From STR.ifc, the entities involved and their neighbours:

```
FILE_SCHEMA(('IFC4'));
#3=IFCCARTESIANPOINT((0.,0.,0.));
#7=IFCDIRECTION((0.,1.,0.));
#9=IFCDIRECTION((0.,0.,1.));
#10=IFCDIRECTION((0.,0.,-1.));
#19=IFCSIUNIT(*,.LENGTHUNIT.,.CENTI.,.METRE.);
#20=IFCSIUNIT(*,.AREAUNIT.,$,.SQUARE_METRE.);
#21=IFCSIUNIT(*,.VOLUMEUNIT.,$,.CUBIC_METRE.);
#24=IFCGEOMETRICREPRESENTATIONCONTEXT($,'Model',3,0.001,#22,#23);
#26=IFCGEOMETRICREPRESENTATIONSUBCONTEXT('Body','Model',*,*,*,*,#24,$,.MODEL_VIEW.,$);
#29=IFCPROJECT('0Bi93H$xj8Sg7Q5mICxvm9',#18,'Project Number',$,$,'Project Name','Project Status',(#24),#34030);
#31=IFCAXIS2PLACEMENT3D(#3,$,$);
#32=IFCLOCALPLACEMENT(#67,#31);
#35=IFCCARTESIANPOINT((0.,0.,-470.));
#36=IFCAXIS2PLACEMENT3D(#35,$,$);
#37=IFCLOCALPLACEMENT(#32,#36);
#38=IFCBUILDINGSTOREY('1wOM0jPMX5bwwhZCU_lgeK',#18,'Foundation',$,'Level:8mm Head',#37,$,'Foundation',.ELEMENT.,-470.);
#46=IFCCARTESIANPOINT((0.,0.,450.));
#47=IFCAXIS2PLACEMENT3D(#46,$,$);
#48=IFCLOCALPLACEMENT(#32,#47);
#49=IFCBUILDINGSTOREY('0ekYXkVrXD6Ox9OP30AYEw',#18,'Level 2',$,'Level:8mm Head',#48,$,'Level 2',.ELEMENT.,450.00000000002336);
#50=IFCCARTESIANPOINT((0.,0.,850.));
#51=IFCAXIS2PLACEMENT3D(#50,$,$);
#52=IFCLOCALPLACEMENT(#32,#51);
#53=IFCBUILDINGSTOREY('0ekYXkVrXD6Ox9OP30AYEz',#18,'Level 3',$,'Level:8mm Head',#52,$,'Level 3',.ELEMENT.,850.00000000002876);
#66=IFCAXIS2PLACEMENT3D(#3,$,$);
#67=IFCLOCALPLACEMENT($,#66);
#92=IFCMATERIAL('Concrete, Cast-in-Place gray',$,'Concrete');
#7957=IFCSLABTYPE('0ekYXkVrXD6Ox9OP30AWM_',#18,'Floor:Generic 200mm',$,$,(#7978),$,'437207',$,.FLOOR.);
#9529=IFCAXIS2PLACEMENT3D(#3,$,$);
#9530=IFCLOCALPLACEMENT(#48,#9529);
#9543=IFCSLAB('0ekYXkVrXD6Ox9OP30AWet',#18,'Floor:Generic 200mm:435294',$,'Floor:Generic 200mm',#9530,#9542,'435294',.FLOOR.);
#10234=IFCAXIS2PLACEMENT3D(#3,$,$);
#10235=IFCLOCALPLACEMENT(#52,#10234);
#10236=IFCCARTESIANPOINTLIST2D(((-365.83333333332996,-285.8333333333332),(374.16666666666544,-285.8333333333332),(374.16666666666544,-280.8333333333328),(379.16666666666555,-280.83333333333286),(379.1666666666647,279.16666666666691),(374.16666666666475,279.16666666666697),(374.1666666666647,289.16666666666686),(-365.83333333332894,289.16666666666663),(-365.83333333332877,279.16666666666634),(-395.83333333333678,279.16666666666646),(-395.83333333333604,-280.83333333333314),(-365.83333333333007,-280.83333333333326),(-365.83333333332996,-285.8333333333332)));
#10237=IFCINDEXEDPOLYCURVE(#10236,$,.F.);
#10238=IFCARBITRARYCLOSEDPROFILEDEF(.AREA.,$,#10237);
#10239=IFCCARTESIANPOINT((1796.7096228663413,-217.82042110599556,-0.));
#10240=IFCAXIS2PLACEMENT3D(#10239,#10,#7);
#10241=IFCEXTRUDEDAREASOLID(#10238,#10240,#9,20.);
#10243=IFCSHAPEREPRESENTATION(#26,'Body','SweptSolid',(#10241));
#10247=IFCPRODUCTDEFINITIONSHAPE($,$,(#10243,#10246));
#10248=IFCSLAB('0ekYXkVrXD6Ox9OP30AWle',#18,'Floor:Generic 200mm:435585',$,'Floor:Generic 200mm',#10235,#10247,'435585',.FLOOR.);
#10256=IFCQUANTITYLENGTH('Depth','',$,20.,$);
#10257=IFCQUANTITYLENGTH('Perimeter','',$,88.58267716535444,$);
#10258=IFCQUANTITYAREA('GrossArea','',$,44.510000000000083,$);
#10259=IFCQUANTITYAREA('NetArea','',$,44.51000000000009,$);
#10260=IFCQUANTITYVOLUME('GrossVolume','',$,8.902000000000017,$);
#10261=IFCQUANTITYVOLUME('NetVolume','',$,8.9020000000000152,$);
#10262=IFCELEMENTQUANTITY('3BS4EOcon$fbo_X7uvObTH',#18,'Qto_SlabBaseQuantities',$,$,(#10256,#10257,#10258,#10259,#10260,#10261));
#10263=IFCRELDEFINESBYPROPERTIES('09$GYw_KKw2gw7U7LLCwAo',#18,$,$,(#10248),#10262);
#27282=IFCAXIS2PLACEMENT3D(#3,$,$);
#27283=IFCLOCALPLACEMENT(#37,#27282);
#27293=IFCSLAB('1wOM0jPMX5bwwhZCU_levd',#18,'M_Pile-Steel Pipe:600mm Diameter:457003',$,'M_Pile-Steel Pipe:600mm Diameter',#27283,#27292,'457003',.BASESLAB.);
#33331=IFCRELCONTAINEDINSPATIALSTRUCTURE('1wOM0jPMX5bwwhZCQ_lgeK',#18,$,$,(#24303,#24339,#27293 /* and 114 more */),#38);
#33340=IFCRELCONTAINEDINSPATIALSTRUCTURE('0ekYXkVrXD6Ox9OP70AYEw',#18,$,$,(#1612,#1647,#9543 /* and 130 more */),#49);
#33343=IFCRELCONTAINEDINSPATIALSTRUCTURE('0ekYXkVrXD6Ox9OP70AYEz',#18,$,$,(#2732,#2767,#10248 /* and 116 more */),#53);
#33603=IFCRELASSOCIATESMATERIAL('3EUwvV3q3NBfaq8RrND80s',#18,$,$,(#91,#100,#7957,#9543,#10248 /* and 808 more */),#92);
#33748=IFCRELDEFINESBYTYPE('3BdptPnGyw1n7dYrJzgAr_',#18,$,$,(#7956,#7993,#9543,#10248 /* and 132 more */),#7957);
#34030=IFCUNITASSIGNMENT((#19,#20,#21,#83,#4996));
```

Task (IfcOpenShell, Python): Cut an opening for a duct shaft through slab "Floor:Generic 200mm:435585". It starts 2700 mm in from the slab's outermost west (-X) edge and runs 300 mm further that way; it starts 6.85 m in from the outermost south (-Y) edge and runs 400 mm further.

```python
import numpy as np
import ifcopenshell
import ifcopenshell.api.feature
import ifcopenshell.api.geometry
import ifcopenshell.api.pset
import ifcopenshell.api.root
import ifcopenshell.geom
import ifcopenshell.util.element
import ifcopenshell.util.placement
import ifcopenshell.util.representation
import ifcopenshell.util.shape
import ifcopenshell.util.unit

model = ifcopenshell.open("STR.ifc")
unit_scale = ifcopenshell.util.unit.calculate_unit_scale(model)
area_scale = ifcopenshell.util.unit.calculate_unit_scale(model, "AREAUNIT")
volume_scale = ifcopenshell.util.unit.calculate_unit_scale(model, "VOLUMEUNIT")
settings = ifcopenshell.geom.settings()


def volume(element):
    """Net volume in cubic metres, openings subtracted."""
    shape = ifcopenshell.geom.create_shape(settings, element)
    return ifcopenshell.util.shape.get_volume(shape.geometry)


slab = model.by_guid("0ekYXkVrXD6Ox9OP30AWle")
before = volume(slab)

# Extent in the slab's own axes, in metres. The edges named are its -X and -Y sides.
slab_shape = ifcopenshell.geom.create_shape(settings, slab)
vertices = ifcopenshell.util.shape.get_vertices(slab_shape.geometry)
x_min, y_min, bottom = vertices.min(axis=0)
top = vertices[:, 2].max()

opening = ifcopenshell.api.root.create_entity(model, ifc_class="IfcOpeningElement", name="Duct shaft opening", predefined_type="OPENING")
context = ifcopenshell.util.representation.get_context(model, "Model", "Body", "MODEL_VIEW")
width, depth = 0.3, 0.4
outline = [(0.0, 0.0), (width, 0.0), (width, depth), (0.0, depth), (0.0, 0.0)]
# Overshoot both faces by 50 mm so the cut is clean.
shape = ifcopenshell.api.geometry.add_slab_representation(
    model, context=context, depth=top - bottom + 0.1, polyline=outline
)
ifcopenshell.api.geometry.assign_representation(model, product=opening, representation=shape)

matrix = ifcopenshell.util.placement.get_local_placement(slab.ObjectPlacement)
matrix[:, 3] = matrix @ np.append(np.array([x_min + 2.7, y_min + 6.85, bottom - 0.05]) / unit_scale, 1.0)
ifcopenshell.api.geometry.edit_object_placement(model, product=opening, matrix=matrix, is_si=False)
ifcopenshell.api.feature.add_feature(model, feature=opening, element=slab)

after = volume(slab)

# Update the slab's stored quantities.
qto = model.by_id(ifcopenshell.util.element.get_pset(slab, "Qto_SlabBaseQuantities", should_inherit=False)["id"])
ifcopenshell.api.pset.edit_qto(model, qto=qto, properties={
    "NetArea": after / (top - bottom) / area_scale,
    "NetVolume": after / volume_scale,
})

print(f"slab volume {before:.3f} -> {after:.3f} m3")

model.write("STR_updated.ifc")
```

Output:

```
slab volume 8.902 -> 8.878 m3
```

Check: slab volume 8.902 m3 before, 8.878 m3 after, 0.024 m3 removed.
